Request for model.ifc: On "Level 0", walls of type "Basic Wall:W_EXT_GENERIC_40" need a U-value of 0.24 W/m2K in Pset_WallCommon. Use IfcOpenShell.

First a look at what the model holds.

```python
import ifcopenshell
import ifcopenshell.util.element

model = ifcopenshell.open("model.ifc")
print(model.schema)
storey = next(s for s in model.by_type("IfcBuildingStorey") if s.Name == "Level 0")
walls = [e for e in ifcopenshell.util.element.get_decomposition(storey) if e.is_a("IfcWall")]
seen = {}
for e in walls:
    element_type = ifcopenshell.util.element.get_type(e)
    key = (element_type.Name if element_type != e and element_type else None, ifcopenshell.util.element.get_pset(e, "Pset_WallCommon", "ThermalTransmittance"))
    seen[key] = seen.get(key, 0) + 1
for (name, value), count in sorted(seen.items(), key=str):
    print(count, "x", name, "|", value)
```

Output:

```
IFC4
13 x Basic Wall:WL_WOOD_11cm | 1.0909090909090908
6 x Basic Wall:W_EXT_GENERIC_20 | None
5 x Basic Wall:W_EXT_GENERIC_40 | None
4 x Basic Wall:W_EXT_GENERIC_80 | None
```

```python
import ifcopenshell
import ifcopenshell.api.pset
import ifcopenshell.util.element

model = ifcopenshell.open("model.ifc")

storey = next(s for s in model.by_type("IfcBuildingStorey") if s.Name == "Level 0")
walls = [e for e in ifcopenshell.util.element.get_decomposition(storey) if e.is_a("IfcWall")]

count = 0
for e in walls:
    element_type = ifcopenshell.util.element.get_type(e)
    if element_type in (None, e) or element_type.Name != "Basic Wall:W_EXT_GENERIC_40":
        continue
    # add_pset returns the element's existing set when there is one.
    pset = ifcopenshell.api.pset.add_pset(model, product=e, name="Pset_WallCommon")
    ifcopenshell.api.pset.edit_pset(model, pset=pset, properties={"ThermalTransmittance": 0.24})
    count += 1

print(count, "walls updated")

model.write("model_updated.ifc")
```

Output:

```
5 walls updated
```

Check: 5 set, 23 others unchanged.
